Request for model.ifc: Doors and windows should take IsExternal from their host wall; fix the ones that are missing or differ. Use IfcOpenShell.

First a look at what the model holds.

```python
import ifcopenshell
import ifcopenshell.util.element

model = ifcopenshell.open("model.ifc")
print(model.schema)
seen = {}
for e in model.by_type("IfcDoor") + model.by_type("IfcWindow"):
    if not e.FillsVoids:
        continue
    host = e.FillsVoids[0].RelatingOpeningElement.VoidsElements[0].RelatingBuildingElement
    own = ifcopenshell.util.element.get_pset(e, f"Pset_{e.is_a()[3:].removesuffix('StandardCase')}Common", "IsExternal")
    wall = ifcopenshell.util.element.get_pset(host, "Pset_WallCommon", "IsExternal")
    seen[e.is_a(), own, wall] = seen.get((e.is_a(), own, wall), 0) + 1
for (cls, own, wall), count in sorted(seen.items(), key=str):
    print(count, cls, "IsExternal:", own, "| host wall:", wall)
```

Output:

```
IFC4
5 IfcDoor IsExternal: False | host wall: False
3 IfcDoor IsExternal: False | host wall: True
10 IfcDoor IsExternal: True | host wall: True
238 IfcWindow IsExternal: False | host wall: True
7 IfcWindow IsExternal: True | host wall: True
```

```python
import ifcopenshell
import ifcopenshell.api.pset
import ifcopenshell.util.element

model = ifcopenshell.open("model.ifc")

count = 0
for ifc_class, pset_name in (("IfcDoor", "Pset_DoorCommon"), ("IfcWindow", "Pset_WindowCommon")):
    for e in model.by_type(ifc_class):
        if not e.FillsVoids:
            continue
        host = e.FillsVoids[0].RelatingOpeningElement.VoidsElements[0].RelatingBuildingElement
        external = ifcopenshell.util.element.get_pset(host, "Pset_WallCommon", "IsExternal")
        if external is None or ifcopenshell.util.element.get_pset(e, pset_name, "IsExternal") == external:
            continue
        pset = ifcopenshell.api.pset.add_pset(model, product=e, name=pset_name)
        ifcopenshell.api.pset.edit_pset(model, pset=pset, properties={"IsExternal": external})
        count += 1

print(count, "updated")

model.write("model_v2.ifc")
```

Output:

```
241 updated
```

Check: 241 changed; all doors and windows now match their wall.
